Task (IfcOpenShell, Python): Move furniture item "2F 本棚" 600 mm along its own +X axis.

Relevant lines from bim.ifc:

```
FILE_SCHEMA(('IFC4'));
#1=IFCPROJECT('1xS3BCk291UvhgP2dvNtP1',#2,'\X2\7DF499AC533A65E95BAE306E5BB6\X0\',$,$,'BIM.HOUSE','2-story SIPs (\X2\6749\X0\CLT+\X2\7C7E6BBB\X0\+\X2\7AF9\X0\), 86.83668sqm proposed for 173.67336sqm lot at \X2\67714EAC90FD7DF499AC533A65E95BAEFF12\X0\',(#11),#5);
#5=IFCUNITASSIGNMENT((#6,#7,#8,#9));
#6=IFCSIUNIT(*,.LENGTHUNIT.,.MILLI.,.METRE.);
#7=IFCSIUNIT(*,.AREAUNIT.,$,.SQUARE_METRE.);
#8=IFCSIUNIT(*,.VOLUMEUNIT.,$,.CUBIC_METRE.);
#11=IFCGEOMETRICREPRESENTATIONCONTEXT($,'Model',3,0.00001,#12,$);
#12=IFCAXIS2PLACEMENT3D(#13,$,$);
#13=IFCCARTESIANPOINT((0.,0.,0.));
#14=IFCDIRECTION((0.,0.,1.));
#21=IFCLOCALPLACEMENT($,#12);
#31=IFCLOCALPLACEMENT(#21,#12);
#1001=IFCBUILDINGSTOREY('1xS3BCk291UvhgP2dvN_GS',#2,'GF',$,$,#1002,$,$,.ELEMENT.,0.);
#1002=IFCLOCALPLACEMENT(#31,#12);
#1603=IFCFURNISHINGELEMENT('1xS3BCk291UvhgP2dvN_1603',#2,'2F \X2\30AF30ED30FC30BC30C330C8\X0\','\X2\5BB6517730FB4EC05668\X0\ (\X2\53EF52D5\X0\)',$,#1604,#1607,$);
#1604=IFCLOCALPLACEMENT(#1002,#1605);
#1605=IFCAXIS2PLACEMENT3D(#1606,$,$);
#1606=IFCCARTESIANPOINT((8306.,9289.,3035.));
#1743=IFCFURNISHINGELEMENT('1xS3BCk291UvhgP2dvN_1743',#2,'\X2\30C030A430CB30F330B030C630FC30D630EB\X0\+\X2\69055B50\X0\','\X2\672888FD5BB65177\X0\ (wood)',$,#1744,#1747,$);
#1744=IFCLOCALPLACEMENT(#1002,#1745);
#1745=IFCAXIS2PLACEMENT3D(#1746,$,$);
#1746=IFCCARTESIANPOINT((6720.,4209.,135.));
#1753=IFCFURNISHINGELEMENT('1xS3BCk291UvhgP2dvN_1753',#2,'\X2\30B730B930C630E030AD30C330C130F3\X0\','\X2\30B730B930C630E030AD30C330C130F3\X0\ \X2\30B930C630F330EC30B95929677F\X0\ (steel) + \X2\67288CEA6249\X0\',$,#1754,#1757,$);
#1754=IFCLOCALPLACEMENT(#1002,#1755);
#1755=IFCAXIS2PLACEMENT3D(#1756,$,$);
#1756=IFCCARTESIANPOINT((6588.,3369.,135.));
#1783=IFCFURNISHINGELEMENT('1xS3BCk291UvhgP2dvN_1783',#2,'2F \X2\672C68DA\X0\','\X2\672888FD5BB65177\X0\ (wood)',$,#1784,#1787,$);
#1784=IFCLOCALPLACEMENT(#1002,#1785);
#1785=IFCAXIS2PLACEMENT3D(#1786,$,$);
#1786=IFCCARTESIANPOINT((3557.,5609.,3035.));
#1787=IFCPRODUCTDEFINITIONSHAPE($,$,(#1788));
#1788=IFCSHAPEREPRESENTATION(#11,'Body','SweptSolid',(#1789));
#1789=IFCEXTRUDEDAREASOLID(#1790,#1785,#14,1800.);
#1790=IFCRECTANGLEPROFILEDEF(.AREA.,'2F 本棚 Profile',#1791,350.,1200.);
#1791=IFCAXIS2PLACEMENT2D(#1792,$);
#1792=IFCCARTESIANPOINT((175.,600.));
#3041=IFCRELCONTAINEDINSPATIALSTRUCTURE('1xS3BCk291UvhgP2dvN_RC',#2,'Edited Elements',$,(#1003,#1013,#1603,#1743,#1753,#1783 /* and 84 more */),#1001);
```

```python
import ifcopenshell
import ifcopenshell.api.geometry
import ifcopenshell.util.placement
import ifcopenshell.util.unit

model = ifcopenshell.open("bim.ifc")
unit_scale = ifcopenshell.util.unit.calculate_unit_scale(model)

item = model.by_guid("1xS3BCk291UvhgP2dvN_1783")
matrix = ifcopenshell.util.placement.get_local_placement(item.ObjectPlacement)
matrix[:3, 3] += matrix[:3, 0] * 0.6 / unit_scale
ifcopenshell.api.geometry.edit_object_placement(model, product=item, matrix=matrix, is_si=False)

print(ifcopenshell.util.placement.get_local_placement(item.ObjectPlacement).round(3) + 0.0)

model.write("bim_rev.ifc")
```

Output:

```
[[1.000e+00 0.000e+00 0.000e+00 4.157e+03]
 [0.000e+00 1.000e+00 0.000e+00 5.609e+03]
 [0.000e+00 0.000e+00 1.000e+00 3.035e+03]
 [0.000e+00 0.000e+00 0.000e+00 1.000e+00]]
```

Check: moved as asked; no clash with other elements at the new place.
